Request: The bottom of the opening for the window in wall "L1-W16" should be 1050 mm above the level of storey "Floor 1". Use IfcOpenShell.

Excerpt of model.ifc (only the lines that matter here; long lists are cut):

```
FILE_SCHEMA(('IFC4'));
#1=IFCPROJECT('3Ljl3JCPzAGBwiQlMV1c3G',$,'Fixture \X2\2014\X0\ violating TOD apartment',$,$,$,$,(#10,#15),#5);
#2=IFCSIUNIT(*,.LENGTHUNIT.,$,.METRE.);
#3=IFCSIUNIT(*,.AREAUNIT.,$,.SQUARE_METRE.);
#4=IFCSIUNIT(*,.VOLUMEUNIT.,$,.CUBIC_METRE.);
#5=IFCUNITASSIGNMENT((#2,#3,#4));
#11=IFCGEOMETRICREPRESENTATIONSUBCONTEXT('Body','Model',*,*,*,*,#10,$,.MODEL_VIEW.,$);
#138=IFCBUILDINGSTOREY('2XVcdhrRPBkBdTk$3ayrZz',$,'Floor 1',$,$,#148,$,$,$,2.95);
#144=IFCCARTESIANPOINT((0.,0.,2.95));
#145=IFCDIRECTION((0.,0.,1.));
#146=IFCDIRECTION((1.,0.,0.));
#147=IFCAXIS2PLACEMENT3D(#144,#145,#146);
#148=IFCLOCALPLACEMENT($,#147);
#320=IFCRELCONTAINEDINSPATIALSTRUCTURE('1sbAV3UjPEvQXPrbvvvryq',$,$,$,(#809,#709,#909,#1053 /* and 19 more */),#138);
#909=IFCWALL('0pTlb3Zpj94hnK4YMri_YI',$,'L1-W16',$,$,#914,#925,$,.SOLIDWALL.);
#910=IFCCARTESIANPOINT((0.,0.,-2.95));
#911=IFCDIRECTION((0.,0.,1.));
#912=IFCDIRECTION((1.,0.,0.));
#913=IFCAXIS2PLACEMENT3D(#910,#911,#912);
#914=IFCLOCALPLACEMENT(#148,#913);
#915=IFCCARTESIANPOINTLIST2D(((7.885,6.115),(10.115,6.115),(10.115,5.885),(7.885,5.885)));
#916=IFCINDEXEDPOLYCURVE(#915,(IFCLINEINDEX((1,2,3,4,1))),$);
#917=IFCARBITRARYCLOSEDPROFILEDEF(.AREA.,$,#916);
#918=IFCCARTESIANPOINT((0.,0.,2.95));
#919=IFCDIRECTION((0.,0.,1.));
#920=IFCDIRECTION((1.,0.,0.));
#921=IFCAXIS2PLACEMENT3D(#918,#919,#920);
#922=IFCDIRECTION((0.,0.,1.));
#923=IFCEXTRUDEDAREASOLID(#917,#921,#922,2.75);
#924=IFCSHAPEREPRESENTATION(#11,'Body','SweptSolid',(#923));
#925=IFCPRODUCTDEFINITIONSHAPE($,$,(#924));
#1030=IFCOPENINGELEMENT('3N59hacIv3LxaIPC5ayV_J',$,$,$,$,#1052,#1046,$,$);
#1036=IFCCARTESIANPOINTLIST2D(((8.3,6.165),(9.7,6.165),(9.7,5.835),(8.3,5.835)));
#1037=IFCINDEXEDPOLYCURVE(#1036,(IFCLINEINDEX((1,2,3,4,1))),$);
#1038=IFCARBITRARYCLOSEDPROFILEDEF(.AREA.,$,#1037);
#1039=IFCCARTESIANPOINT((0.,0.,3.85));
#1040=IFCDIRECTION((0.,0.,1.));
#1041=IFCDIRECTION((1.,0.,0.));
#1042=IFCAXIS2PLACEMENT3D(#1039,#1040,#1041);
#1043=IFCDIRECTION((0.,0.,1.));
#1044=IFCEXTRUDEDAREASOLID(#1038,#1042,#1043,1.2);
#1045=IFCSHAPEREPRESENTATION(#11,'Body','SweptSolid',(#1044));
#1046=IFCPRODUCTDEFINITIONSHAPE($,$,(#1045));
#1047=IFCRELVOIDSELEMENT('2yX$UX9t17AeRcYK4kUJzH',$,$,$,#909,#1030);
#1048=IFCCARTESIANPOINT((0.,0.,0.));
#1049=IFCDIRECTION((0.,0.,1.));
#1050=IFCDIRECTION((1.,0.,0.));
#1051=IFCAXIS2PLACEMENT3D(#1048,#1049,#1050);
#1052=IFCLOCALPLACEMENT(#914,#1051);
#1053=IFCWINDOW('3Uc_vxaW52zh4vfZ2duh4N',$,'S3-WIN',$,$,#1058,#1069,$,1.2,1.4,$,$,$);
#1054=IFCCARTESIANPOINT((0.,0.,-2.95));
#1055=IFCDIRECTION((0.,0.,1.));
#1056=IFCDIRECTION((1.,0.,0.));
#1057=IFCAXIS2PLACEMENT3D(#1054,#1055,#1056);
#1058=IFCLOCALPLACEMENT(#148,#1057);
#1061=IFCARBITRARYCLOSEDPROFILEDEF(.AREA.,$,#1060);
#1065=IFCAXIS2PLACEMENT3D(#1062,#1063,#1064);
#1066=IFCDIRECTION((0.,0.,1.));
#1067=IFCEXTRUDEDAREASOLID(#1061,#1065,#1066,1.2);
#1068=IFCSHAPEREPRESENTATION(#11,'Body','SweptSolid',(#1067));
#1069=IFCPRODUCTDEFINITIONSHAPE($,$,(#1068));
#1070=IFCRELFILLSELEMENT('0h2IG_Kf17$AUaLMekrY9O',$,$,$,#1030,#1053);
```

```python
import numpy as np
import ifcopenshell
import ifcopenshell.api.geometry
import ifcopenshell.geom
import ifcopenshell.util.element
import ifcopenshell.util.placement
import ifcopenshell.util.shape
import ifcopenshell.util.unit

model = ifcopenshell.open("model.ifc")
unit_scale = ifcopenshell.util.unit.calculate_unit_scale(model)

window = model.by_guid("3Uc_vxaW52zh4vfZ2duh4N")
opening = window.FillsVoids[0].RelatingOpeningElement
storey = ifcopenshell.util.element.get_container(window, ifc_class="IfcBuildingStorey")
level = ifcopenshell.util.placement.get_local_placement(storey.ObjectPlacement)[2, 3]

# The opening's origin need not be at the sill, so measure its lowest point.
shape = ifcopenshell.geom.create_shape(ifcopenshell.geom.settings(), opening)
bottom = ifcopenshell.util.shape.get_shape_bottom_elevation(shape, shape.geometry) / unit_scale
dz = level + 1.05 / unit_scale - bottom

shift = np.array([0.0, 0.0, dz])
# The window is not placed relative to its opening, so move both.
for product in (opening, window):
    matrix = ifcopenshell.util.placement.get_local_placement(product.ObjectPlacement)
    matrix[:3, 3] += shift
    ifcopenshell.api.geometry.edit_object_placement(model, product=product, matrix=matrix, is_si=False)

print(f"moved by {dz * unit_scale:+.3f} m")

model.write("model_updated.ifc")
```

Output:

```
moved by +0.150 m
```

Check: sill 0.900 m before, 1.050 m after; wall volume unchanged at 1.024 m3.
